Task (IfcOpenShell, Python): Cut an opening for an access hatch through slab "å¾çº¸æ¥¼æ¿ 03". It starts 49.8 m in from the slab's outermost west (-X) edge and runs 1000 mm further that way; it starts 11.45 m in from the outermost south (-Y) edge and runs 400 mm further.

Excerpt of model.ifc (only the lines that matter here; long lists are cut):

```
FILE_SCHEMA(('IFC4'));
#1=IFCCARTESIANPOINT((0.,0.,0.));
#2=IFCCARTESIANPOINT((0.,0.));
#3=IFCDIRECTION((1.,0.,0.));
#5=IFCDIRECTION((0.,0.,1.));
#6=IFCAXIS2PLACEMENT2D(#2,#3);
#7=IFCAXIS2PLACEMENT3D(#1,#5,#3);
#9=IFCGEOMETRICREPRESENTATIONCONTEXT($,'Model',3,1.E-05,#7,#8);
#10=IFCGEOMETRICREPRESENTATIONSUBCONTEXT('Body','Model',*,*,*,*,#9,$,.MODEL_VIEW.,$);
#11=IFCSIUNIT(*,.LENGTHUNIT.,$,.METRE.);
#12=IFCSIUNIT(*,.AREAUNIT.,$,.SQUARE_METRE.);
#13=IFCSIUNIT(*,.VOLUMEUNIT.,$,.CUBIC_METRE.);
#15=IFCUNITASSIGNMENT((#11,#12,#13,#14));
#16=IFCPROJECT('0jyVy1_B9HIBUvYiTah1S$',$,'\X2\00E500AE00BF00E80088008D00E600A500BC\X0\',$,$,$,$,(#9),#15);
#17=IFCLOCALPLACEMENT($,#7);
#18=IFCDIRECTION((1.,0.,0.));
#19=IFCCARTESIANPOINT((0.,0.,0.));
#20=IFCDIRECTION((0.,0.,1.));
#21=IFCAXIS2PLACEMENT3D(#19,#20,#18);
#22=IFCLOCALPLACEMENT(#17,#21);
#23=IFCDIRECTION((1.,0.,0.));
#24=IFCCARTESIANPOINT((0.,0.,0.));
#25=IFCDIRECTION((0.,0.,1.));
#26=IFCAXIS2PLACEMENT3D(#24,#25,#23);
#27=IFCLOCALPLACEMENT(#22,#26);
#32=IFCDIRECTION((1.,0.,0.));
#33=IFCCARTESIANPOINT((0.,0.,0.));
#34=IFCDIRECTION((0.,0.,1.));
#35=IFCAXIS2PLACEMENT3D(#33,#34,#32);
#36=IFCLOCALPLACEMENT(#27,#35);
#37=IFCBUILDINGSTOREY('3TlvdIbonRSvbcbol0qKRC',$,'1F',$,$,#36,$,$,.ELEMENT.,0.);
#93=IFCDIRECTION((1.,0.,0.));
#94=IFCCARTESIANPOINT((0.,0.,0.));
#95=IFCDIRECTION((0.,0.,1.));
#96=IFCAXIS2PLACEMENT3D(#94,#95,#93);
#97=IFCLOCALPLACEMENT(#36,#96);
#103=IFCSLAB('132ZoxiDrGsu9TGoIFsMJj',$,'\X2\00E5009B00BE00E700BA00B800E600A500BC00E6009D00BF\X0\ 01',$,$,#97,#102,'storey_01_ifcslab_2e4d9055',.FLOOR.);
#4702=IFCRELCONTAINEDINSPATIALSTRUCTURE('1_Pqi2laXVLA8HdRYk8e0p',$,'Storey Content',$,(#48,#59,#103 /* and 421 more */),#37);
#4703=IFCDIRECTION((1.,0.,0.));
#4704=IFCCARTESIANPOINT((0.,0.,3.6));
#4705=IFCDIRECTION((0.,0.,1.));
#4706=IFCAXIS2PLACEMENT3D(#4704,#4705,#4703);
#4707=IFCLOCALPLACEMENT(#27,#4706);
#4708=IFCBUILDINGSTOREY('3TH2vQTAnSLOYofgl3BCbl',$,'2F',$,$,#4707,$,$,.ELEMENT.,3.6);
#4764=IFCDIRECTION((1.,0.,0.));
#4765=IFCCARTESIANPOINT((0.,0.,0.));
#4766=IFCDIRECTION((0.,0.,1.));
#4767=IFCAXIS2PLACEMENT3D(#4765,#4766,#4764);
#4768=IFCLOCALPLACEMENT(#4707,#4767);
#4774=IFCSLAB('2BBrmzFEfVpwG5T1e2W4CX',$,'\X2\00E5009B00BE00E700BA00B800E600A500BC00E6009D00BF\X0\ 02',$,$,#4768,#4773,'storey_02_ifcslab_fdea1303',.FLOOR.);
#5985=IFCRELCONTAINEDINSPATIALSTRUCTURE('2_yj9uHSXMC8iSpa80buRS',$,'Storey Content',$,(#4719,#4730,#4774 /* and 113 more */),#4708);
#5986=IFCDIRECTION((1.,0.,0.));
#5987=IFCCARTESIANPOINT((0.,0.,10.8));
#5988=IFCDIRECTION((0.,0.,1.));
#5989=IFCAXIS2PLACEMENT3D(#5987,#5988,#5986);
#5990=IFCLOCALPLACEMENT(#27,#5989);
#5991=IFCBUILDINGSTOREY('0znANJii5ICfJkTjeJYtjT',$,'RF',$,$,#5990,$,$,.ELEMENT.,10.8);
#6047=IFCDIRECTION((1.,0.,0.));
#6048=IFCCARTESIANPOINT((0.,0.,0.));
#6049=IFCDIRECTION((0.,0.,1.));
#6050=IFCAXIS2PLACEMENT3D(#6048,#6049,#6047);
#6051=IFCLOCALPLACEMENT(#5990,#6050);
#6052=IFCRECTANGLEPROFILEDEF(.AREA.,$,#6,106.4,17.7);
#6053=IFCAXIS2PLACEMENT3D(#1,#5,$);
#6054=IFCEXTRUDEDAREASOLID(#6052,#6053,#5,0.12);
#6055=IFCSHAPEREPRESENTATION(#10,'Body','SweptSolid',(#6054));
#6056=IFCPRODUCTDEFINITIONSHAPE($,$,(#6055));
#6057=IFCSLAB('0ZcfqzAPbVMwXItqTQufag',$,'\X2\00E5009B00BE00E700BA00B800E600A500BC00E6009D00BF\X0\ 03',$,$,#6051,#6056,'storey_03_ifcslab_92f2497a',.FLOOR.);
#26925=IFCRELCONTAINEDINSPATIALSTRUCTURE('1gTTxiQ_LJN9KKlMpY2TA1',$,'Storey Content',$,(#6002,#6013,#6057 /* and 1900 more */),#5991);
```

```python
import numpy as np
import ifcopenshell
import ifcopenshell.api.feature
import ifcopenshell.api.geometry
import ifcopenshell.api.root
import ifcopenshell.geom
import ifcopenshell.util.placement
import ifcopenshell.util.representation
import ifcopenshell.util.shape
import ifcopenshell.util.unit

model = ifcopenshell.open("model.ifc")
unit_scale = ifcopenshell.util.unit.calculate_unit_scale(model)
settings = ifcopenshell.geom.settings()


def volume(element):
    """Net volume in cubic metres, openings subtracted."""
    shape = ifcopenshell.geom.create_shape(settings, element)
    return ifcopenshell.util.shape.get_volume(shape.geometry)


slab = model.by_id(6057)
before = volume(slab)

# Extent in the slab's own axes, in metres. The edges named are its -X and -Y sides.
slab_shape = ifcopenshell.geom.create_shape(settings, slab)
vertices = ifcopenshell.util.shape.get_vertices(slab_shape.geometry)
x_min, y_min, bottom = vertices.min(axis=0)
top = vertices[:, 2].max()

opening = ifcopenshell.api.root.create_entity(model, ifc_class="IfcOpeningElement", name="Access hatch opening", predefined_type="OPENING")
context = ifcopenshell.util.representation.get_context(model, "Model", "Body", "MODEL_VIEW")
width, depth = 1, 0.4
outline = [(0.0, 0.0), (width, 0.0), (width, depth), (0.0, depth), (0.0, 0.0)]
# Overshoot both faces by 50 mm so the cut is clean.
shape = ifcopenshell.api.geometry.add_slab_representation(
    model, context=context, depth=top - bottom + 0.1, polyline=outline
)
ifcopenshell.api.geometry.assign_representation(model, product=opening, representation=shape)

matrix = ifcopenshell.util.placement.get_local_placement(slab.ObjectPlacement)
matrix[:, 3] = matrix @ np.append(np.array([x_min + 49.8, y_min + 11.45, bottom - 0.05]) / unit_scale, 1.0)
ifcopenshell.api.geometry.edit_object_placement(model, product=opening, matrix=matrix, is_si=False)
ifcopenshell.api.feature.add_feature(model, feature=opening, element=slab)

after = volume(slab)

print(f"slab volume {before:.3f} -> {after:.3f} m3")

model.write("model_v2.ifc")
```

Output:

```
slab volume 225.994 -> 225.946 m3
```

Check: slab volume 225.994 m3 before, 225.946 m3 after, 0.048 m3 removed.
